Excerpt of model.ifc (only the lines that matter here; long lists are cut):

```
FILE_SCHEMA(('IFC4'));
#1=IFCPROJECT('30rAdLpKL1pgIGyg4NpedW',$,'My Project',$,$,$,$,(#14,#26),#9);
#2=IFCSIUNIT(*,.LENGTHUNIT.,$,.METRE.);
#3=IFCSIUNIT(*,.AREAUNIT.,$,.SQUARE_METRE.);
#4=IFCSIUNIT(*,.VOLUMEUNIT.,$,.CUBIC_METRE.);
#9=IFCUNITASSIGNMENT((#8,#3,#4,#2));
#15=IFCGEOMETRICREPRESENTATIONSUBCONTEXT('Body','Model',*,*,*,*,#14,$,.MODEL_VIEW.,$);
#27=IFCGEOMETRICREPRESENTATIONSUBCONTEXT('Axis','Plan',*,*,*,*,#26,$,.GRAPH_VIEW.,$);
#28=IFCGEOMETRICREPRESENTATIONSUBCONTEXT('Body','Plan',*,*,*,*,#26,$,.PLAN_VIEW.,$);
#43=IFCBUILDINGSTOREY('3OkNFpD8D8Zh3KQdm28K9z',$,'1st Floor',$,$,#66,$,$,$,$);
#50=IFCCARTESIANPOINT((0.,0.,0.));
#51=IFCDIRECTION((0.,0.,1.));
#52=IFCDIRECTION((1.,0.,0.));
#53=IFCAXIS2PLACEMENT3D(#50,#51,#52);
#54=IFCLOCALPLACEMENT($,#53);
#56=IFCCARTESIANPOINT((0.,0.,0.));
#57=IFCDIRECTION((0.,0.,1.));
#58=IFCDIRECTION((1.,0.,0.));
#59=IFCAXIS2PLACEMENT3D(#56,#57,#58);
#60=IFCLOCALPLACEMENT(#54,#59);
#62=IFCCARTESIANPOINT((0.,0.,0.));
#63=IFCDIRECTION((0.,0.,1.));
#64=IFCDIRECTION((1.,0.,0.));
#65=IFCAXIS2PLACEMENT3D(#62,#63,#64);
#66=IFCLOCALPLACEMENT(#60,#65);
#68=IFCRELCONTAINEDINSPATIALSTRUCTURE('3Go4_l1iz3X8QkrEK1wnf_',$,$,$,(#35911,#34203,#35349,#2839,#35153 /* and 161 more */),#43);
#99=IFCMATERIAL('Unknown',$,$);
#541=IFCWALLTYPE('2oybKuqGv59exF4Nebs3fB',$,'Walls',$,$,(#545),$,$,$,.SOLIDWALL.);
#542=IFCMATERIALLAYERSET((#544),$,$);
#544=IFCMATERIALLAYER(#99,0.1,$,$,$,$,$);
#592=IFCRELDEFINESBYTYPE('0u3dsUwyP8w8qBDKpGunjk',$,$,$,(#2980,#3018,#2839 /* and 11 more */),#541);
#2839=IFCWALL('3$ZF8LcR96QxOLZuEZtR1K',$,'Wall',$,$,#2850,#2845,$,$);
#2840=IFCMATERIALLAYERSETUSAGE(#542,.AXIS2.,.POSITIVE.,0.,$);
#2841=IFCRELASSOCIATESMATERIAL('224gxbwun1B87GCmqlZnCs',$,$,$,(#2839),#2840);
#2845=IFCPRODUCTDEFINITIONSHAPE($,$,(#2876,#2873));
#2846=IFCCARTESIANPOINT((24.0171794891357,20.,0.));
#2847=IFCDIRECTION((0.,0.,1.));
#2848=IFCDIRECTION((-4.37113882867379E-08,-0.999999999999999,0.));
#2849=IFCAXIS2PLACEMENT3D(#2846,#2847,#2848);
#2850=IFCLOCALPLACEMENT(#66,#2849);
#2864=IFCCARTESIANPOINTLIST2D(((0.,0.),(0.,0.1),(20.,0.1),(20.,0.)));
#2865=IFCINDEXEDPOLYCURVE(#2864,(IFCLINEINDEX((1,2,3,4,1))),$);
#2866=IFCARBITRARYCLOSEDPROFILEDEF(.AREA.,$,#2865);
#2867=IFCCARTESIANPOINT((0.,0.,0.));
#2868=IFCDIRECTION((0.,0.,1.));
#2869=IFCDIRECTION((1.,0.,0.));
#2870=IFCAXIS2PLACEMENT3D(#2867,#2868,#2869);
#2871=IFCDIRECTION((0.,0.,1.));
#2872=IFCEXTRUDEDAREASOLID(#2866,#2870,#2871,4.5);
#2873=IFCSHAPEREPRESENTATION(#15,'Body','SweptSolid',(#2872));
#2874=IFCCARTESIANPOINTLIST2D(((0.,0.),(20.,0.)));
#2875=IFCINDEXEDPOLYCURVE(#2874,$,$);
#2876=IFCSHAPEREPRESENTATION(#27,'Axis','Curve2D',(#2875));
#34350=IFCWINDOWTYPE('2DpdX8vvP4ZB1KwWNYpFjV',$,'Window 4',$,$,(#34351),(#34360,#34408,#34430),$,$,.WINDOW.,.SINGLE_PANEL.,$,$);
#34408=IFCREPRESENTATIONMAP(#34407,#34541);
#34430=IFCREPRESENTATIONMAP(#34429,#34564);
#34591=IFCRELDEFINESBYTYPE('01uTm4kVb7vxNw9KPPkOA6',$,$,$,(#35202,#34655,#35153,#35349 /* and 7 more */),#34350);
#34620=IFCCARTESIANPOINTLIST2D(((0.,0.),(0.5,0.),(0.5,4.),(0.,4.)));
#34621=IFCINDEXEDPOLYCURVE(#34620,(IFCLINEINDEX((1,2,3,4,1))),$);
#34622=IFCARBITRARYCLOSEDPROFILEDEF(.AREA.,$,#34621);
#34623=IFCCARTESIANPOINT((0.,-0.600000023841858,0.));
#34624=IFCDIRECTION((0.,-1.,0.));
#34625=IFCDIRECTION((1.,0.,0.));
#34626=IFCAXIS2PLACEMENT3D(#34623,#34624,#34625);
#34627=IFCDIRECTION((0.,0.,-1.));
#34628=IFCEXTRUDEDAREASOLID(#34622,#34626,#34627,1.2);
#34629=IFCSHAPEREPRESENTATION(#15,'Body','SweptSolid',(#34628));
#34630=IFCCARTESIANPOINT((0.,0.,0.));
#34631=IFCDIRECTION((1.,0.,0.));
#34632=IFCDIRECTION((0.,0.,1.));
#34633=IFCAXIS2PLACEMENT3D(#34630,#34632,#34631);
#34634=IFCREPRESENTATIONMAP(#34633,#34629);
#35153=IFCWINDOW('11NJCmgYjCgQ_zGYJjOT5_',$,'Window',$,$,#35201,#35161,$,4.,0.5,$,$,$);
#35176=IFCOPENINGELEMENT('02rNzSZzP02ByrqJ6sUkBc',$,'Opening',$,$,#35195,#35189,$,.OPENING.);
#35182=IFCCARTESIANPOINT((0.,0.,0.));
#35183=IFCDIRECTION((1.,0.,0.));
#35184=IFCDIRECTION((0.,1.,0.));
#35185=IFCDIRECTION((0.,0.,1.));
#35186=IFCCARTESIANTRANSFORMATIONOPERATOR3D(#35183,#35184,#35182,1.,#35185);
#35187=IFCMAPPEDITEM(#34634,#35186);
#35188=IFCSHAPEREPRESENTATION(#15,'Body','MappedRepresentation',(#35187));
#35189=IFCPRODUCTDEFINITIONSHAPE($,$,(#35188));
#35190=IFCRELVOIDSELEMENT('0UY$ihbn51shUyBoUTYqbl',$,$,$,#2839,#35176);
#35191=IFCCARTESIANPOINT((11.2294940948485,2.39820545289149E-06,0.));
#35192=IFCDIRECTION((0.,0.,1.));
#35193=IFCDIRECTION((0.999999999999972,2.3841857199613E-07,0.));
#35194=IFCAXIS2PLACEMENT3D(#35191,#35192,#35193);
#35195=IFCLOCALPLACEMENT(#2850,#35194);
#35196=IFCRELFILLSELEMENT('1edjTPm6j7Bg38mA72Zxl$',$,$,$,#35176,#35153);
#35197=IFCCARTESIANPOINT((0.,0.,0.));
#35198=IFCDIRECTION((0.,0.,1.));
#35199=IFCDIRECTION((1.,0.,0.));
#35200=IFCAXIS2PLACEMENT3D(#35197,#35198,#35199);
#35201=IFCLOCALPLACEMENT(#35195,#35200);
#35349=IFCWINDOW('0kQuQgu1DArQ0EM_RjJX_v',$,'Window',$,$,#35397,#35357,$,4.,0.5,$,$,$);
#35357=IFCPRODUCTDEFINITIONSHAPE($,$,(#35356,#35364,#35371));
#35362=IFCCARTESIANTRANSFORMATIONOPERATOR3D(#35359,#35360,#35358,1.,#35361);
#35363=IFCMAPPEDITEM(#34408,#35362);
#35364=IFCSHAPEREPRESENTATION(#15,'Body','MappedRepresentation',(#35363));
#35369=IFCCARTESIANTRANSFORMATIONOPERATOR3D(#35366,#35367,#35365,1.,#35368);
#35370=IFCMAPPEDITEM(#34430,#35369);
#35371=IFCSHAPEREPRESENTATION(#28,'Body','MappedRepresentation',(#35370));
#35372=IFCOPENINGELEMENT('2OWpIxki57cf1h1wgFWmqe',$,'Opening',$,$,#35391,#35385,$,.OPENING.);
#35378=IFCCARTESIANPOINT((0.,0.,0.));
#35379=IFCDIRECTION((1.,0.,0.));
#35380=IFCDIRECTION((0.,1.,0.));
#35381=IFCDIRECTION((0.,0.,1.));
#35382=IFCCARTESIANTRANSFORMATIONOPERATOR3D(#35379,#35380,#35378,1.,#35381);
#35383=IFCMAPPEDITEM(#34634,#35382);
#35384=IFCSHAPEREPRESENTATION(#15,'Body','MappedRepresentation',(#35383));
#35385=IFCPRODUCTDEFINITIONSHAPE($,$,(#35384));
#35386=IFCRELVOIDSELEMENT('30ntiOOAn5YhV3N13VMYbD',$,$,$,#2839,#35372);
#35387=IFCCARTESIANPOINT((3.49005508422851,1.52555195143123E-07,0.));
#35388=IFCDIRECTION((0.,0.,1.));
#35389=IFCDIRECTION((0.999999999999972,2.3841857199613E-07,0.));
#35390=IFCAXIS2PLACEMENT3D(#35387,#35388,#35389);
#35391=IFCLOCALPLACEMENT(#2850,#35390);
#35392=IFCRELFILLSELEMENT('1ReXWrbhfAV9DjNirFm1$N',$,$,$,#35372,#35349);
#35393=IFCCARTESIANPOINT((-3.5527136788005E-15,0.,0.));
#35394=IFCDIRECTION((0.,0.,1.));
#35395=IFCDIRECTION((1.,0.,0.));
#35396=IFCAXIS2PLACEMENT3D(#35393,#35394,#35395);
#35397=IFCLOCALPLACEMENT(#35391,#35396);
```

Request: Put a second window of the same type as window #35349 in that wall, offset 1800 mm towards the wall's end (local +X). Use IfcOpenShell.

```python
import ifcopenshell
import ifcopenshell.api.feature
import ifcopenshell.api.geometry
import ifcopenshell.api.root
import ifcopenshell.geom
import ifcopenshell.util.element
import ifcopenshell.util.placement
import ifcopenshell.util.shape

model = ifcopenshell.open("model.ifc")
settings = ifcopenshell.geom.settings()


def volume(element):
    """Net volume in cubic metres, openings subtracted."""
    shape = ifcopenshell.geom.create_shape(settings, element)
    return ifcopenshell.util.shape.get_volume(shape.geometry)


window = model.by_guid("0kQuQgu1DArQ0EM_RjJX_v")
opening = window.FillsVoids[0].RelatingOpeningElement
wall = opening.VoidsElements[0].RelatingBuildingElement
before = volume(wall)
shift = ifcopenshell.util.placement.get_local_placement(wall.ObjectPlacement)[:3, 0] * 1.8

# copy_class copies the void relationship, type, container and properties, but no geometry.
new_opening = ifcopenshell.api.root.copy_class(model, product=opening)
new_opening.Representation = ifcopenshell.util.element.copy_deep(
    model, opening.Representation, exclude=["IfcGeometricRepresentationContext", "IfcRepresentationMap"]
)
new_window = ifcopenshell.api.root.copy_class(model, product=window)
new_window.Representation = ifcopenshell.util.element.copy_deep(
    model, window.Representation, exclude=["IfcGeometricRepresentationContext", "IfcRepresentationMap"]
)
ifcopenshell.api.feature.add_filling(model, opening=new_opening, element=new_window)

for old, new in ((opening, new_opening), (window, new_window)):
    matrix = ifcopenshell.util.placement.get_local_placement(old.ObjectPlacement)
    matrix[:3, 3] += shift
    ifcopenshell.api.geometry.edit_object_placement(model, product=new, matrix=matrix, is_si=False)

after = volume(wall)

print(f"wall volume {before:.3f} -> {after:.3f} m3")

model.write("model_v2.ifc")
```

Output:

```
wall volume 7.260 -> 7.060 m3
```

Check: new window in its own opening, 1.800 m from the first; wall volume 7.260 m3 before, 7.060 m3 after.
